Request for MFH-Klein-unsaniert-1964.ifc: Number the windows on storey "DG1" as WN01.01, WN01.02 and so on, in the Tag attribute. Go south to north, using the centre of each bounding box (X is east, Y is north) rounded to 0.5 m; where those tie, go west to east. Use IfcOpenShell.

First a look at what the model holds.

```python
import ifcopenshell
import ifcopenshell.util.element
import ifcopenshell.util.placement

model = ifcopenshell.open("MFH-Klein-unsaniert-1964.ifc")
print(model.schema)
storey = next(s for s in model.by_type("IfcBuildingStorey") if s.Name == "DG1")
windows = [e for e in ifcopenshell.util.element.get_decomposition(storey) if e.is_a("IfcWindow")]
for e in sorted(windows, key=lambda e: e.id()):
    origin = ifcopenshell.util.placement.get_local_placement(e.ObjectPlacement)[:3, 3]
    print(e.id(), e.Tag, e.Name, origin.round(2) + 0.0, sep=" | ")
```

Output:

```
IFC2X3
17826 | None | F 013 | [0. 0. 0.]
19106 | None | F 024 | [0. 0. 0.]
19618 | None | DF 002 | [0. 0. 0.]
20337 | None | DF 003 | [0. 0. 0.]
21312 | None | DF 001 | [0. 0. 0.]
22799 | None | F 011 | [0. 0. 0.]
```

```python
import ifcopenshell
import ifcopenshell.geom
import ifcopenshell.util.element
import ifcopenshell.util.shape

model = ifcopenshell.open("MFH-Klein-unsaniert-1964.ifc")
settings = ifcopenshell.geom.settings()
settings.set("use-world-coords", True)


def centre(element):
    shape = ifcopenshell.geom.create_shape(settings, element)
    return ifcopenshell.util.shape.get_bbox_centroid(shape.geometry)


storey = next(s for s in model.by_type("IfcBuildingStorey") if s.Name == "DG1")
windows = [e for e in ifcopenshell.util.element.get_decomposition(storey) if e.is_a("IfcWindow")]

# Insertion points can sit at a corner or the storey origin, so sort by the geometry (in metres).
centres = {e: centre(e) for e in windows}
windows.sort(key=lambda e: (round(centres[e][1] / 0.5), centres[e][0]))

for i, e in enumerate(windows, start=1):
    number = f"WN01.{i:02d}"
    e.Tag = number
    print(e.id(), number)

model.write("MFH-Klein-unsaniert-1964_rev.ifc")
```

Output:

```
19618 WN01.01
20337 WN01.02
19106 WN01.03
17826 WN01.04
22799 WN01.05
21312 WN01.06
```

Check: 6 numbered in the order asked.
